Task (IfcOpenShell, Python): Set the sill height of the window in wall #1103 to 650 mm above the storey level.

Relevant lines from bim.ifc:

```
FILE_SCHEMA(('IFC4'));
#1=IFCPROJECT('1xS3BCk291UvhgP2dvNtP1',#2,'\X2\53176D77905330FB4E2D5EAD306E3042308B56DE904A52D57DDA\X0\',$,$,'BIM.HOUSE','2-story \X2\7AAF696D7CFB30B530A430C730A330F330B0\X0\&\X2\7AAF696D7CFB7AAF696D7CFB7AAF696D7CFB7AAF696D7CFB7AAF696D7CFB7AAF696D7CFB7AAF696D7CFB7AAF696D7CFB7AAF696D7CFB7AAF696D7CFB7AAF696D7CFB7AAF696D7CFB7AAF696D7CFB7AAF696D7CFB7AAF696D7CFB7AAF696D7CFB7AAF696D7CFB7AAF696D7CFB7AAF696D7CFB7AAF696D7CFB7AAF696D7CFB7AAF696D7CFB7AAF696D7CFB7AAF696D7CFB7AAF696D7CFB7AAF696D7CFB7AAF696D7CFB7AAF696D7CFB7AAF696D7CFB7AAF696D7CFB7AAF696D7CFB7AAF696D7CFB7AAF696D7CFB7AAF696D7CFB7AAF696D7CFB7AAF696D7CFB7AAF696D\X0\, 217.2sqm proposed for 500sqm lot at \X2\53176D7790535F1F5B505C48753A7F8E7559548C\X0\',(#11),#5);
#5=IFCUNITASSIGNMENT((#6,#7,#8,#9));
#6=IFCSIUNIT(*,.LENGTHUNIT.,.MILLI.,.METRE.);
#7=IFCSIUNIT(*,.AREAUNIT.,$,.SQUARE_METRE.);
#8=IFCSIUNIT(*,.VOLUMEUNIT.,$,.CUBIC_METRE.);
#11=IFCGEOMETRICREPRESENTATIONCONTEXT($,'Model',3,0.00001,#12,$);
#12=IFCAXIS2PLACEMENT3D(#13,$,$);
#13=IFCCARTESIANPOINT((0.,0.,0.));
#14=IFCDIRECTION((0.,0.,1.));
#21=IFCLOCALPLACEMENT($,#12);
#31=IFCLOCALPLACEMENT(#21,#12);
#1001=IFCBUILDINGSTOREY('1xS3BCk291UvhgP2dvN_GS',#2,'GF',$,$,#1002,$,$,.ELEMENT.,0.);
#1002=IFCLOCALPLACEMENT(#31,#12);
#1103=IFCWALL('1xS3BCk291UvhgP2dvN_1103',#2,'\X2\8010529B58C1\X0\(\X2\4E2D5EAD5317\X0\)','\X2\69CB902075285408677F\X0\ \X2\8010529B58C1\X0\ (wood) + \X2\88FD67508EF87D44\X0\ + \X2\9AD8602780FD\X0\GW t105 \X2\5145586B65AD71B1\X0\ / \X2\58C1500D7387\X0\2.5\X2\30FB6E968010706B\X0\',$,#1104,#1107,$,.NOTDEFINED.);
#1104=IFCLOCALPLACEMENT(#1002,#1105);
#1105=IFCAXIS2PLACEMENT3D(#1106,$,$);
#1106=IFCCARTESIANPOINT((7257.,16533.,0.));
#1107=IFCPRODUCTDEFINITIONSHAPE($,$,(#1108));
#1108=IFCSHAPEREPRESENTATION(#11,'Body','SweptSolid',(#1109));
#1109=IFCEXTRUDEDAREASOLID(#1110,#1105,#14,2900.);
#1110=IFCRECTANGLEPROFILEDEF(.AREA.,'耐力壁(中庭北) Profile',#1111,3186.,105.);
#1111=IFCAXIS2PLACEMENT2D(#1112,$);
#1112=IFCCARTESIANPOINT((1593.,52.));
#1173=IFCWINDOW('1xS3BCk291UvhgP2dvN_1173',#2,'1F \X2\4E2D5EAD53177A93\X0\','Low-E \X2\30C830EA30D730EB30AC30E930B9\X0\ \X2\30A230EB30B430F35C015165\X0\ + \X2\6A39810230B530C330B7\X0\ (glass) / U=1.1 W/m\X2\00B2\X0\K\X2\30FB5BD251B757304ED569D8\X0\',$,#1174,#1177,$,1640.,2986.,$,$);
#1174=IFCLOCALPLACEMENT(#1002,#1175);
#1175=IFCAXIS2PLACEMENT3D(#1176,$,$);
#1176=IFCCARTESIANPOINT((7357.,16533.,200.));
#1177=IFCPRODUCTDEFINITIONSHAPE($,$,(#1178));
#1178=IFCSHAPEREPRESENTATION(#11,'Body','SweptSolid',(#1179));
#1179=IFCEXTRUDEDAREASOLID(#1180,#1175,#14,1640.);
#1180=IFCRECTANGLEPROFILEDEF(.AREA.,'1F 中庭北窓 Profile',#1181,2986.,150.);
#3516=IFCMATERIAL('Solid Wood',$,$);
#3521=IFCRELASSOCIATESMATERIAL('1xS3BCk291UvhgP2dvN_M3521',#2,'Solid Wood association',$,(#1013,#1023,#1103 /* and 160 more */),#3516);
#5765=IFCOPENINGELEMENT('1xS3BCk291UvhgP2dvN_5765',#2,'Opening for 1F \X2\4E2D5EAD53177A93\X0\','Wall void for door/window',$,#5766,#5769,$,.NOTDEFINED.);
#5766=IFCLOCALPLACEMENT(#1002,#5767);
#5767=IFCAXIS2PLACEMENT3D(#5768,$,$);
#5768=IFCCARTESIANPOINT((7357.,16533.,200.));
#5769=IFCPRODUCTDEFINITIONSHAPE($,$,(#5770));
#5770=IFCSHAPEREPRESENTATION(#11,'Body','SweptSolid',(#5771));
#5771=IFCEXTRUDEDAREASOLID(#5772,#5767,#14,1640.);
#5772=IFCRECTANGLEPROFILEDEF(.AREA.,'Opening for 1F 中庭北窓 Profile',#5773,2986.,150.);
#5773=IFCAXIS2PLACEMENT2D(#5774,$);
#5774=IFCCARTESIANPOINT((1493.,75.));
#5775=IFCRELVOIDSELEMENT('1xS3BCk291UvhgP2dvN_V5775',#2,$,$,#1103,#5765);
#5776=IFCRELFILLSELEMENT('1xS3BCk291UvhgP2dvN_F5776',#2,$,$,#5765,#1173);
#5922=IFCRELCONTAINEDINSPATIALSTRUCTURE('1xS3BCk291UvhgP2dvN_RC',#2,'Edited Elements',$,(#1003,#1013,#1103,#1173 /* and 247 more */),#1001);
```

```python
import numpy as np
import ifcopenshell
import ifcopenshell.api.geometry
import ifcopenshell.geom
import ifcopenshell.util.element
import ifcopenshell.util.placement
import ifcopenshell.util.shape
import ifcopenshell.util.unit

model = ifcopenshell.open("bim.ifc")
unit_scale = ifcopenshell.util.unit.calculate_unit_scale(model)

window = model.by_id(1173)
opening = window.FillsVoids[0].RelatingOpeningElement
storey = ifcopenshell.util.element.get_container(window, ifc_class="IfcBuildingStorey")
level = ifcopenshell.util.placement.get_local_placement(storey.ObjectPlacement)[2, 3]

# The opening's origin need not be at the sill, so measure its lowest point.
shape = ifcopenshell.geom.create_shape(ifcopenshell.geom.settings(), opening)
bottom = ifcopenshell.util.shape.get_shape_bottom_elevation(shape, shape.geometry) / unit_scale
dz = level + 650.0 - bottom

shift = np.array([0.0, 0.0, dz])
# The window is not placed relative to its opening, so move both.
for product in (opening, window):
    matrix = ifcopenshell.util.placement.get_local_placement(product.ObjectPlacement)
    matrix[:3, 3] += shift
    ifcopenshell.api.geometry.edit_object_placement(model, product=product, matrix=matrix, is_si=False)

print(f"moved by {dz * unit_scale:+.3f} m")

model.write("bim_updated.ifc")
```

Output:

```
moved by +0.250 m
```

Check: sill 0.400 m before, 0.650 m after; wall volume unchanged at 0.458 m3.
